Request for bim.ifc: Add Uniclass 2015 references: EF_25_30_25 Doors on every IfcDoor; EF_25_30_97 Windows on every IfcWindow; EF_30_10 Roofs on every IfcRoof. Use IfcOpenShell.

First a look at what the model holds.

```python
import ifcopenshell

model = ifcopenshell.open("bim.ifc")
print(model.schema)
print("classifications:", [c.Name for c in model.by_type("IfcClassification")])
for ifc_class in ("IfcDoor", "IfcRoof", "IfcStair", "IfcWall", "IfcWindow"):
    print(ifc_class, len(model.by_type(ifc_class)))
```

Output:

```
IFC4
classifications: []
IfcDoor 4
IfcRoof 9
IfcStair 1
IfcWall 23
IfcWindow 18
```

```python
import ifcopenshell
import ifcopenshell.api.classification

model = ifcopenshell.open("bim.ifc")

system = ifcopenshell.api.classification.add_classification(model, classification="Uniclass 2015")

codes = {
    "IfcDoor": ("EF_25_30_25", "Doors"),
    "IfcWindow": ("EF_25_30_97", "Windows"),
    "IfcRoof": ("EF_30_10", "Roofs"),
}
for ifc_class, (code, name) in codes.items():
    products = model.by_type(ifc_class)
    ifcopenshell.api.classification.add_reference(
        model, products=products, classification=system, identification=code, name=name
    )
    print(code, len(products))

model.write("bim_edited.ifc")
```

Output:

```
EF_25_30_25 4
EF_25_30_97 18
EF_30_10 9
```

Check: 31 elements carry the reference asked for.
